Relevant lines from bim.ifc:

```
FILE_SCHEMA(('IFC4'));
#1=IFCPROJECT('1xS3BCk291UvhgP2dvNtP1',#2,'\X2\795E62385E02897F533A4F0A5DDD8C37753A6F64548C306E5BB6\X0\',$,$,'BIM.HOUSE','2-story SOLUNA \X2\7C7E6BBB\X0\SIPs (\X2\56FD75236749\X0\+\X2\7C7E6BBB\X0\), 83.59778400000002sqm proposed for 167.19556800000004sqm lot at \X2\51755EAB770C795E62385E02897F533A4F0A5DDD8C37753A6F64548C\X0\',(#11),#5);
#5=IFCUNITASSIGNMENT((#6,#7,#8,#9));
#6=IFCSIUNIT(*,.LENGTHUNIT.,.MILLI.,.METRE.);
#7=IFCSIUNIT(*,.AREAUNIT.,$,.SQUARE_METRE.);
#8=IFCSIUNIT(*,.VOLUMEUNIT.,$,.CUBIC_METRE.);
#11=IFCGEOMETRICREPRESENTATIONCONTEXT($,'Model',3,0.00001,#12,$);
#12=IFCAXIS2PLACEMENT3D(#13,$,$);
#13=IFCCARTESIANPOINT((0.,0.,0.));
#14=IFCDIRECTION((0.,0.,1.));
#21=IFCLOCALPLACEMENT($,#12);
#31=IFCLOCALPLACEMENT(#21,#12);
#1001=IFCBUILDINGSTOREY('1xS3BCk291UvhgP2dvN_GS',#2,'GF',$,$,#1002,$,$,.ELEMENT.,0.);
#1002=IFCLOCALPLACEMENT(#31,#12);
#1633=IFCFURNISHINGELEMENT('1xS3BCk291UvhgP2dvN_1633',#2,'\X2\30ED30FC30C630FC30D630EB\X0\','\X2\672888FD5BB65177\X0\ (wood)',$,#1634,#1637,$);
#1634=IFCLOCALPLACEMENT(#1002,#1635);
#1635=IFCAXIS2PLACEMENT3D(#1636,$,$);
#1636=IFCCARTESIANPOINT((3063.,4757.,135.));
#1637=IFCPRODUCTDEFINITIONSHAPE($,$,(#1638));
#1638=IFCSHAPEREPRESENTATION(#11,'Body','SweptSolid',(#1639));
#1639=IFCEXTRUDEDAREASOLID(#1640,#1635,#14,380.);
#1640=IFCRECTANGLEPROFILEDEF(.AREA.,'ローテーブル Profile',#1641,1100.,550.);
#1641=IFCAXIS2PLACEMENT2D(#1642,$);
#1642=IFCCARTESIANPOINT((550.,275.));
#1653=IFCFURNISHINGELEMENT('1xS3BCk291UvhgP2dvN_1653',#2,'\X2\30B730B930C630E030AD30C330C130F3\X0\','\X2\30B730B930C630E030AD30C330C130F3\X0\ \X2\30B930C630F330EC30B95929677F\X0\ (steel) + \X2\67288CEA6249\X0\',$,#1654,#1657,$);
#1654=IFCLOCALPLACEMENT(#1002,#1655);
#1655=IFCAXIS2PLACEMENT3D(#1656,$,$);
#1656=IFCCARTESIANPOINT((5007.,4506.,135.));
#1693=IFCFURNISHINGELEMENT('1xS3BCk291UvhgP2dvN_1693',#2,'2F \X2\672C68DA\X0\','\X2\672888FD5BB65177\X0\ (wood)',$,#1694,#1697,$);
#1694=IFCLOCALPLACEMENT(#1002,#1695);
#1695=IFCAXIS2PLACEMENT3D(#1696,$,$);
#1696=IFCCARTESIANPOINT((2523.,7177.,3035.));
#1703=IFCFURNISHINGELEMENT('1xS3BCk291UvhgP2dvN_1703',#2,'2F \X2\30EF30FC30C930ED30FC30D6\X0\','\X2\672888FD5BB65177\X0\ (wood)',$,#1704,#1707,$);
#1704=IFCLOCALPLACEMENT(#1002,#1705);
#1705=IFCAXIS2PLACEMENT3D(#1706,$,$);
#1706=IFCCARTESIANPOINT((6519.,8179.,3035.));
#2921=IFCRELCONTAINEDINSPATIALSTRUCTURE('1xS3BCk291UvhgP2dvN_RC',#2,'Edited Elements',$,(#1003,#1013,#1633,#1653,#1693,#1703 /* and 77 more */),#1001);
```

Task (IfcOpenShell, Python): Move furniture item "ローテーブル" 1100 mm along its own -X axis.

```python
import ifcopenshell
import ifcopenshell.api.geometry
import ifcopenshell.util.placement
import ifcopenshell.util.unit

model = ifcopenshell.open("bim.ifc")
unit_scale = ifcopenshell.util.unit.calculate_unit_scale(model)

item = model.by_id(1633)
matrix = ifcopenshell.util.placement.get_local_placement(item.ObjectPlacement)
matrix[:3, 3] -= matrix[:3, 0] * 1.1 / unit_scale
ifcopenshell.api.geometry.edit_object_placement(model, product=item, matrix=matrix, is_si=False)

print(ifcopenshell.util.placement.get_local_placement(item.ObjectPlacement).round(3) + 0.0)

model.write("bim-out.ifc")
```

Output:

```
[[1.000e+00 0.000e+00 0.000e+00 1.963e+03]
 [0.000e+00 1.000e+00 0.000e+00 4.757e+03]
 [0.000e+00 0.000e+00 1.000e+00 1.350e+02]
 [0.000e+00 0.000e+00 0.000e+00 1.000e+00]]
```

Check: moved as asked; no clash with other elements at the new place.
